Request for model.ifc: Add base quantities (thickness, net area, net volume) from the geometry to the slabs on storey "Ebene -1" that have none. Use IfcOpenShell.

First a look at what the model holds.

```python
import ifcopenshell
import ifcopenshell.util.element
import ifcopenshell.util.unit

model = ifcopenshell.open("model.ifc")
print(model.schema)
for unit_type in ("LENGTHUNIT", "AREAUNIT", "VOLUMEUNIT"):
    print(unit_type, ifcopenshell.util.unit.calculate_unit_scale(model, unit_type))
storey = next(s for s in model.by_type("IfcBuildingStorey") if s.Name == "Ebene -1")
slabs = [e for e in ifcopenshell.util.element.get_decomposition(storey) if e.is_a("IfcSlab")]
for e in sorted(slabs, key=lambda e: e.id()):
    print(e.id(), e.is_a(), e.Name, list(ifcopenshell.util.element.get_psets(e, qtos_only=True)), sep=" | ")
```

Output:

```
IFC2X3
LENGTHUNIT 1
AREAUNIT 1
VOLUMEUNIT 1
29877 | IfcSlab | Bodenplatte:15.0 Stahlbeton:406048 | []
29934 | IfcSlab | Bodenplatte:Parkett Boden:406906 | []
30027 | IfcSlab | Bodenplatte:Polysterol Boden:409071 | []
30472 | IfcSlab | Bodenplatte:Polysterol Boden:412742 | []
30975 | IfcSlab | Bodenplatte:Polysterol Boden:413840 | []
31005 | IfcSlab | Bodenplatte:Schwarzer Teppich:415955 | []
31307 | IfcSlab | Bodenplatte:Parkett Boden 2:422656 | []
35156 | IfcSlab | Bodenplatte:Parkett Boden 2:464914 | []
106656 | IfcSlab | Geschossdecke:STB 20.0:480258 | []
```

```python
import ifcopenshell
import ifcopenshell.api.pset
import ifcopenshell.geom
import ifcopenshell.util.element
import ifcopenshell.util.shape
import ifcopenshell.util.unit

model = ifcopenshell.open("model.ifc")
unit_scale = ifcopenshell.util.unit.calculate_unit_scale(model)
area_scale = ifcopenshell.util.unit.calculate_unit_scale(model, "AREAUNIT")
volume_scale = ifcopenshell.util.unit.calculate_unit_scale(model, "VOLUMEUNIT")
settings = ifcopenshell.geom.settings()

storey = next(s for s in model.by_type("IfcBuildingStorey") if s.Name == "Ebene -1")
slabs = [e for e in ifcopenshell.util.element.get_decomposition(storey) if e.is_a("IfcSlab")]

for e in sorted(slabs, key=lambda e: e.id()):
    if ifcopenshell.util.element.get_psets(e, qtos_only=True, should_inherit=False):
        continue
    # Geometry comes back in metres, in the element's own axes.
    shape = ifcopenshell.geom.create_shape(settings, e)
    values = {
        "Width": ifcopenshell.util.shape.get_z(shape.geometry) / unit_scale,
        "NetArea": ifcopenshell.util.shape.get_footprint_area(shape.geometry) / area_scale,
        "NetVolume": ifcopenshell.util.shape.get_volume(shape.geometry) / volume_scale,
    }
    qto = ifcopenshell.api.pset.add_qto(model, product=e, name="BaseQuantities")
    ifcopenshell.api.pset.edit_qto(model, qto=qto, properties=values)
    print(e.id(), {k: round(v, 3) for k, v in values.items()})

model.write("model-out.ifc")
```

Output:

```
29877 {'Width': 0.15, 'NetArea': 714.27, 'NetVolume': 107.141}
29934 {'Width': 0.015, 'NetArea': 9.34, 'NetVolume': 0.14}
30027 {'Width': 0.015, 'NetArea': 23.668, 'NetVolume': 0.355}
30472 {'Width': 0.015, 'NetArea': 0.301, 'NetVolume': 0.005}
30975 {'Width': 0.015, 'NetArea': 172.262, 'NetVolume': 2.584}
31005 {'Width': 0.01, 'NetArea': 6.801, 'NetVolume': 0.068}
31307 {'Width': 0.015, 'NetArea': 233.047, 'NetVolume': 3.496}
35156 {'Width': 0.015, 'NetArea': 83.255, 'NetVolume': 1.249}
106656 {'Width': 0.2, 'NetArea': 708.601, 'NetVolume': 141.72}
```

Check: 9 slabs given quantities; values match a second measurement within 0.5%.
